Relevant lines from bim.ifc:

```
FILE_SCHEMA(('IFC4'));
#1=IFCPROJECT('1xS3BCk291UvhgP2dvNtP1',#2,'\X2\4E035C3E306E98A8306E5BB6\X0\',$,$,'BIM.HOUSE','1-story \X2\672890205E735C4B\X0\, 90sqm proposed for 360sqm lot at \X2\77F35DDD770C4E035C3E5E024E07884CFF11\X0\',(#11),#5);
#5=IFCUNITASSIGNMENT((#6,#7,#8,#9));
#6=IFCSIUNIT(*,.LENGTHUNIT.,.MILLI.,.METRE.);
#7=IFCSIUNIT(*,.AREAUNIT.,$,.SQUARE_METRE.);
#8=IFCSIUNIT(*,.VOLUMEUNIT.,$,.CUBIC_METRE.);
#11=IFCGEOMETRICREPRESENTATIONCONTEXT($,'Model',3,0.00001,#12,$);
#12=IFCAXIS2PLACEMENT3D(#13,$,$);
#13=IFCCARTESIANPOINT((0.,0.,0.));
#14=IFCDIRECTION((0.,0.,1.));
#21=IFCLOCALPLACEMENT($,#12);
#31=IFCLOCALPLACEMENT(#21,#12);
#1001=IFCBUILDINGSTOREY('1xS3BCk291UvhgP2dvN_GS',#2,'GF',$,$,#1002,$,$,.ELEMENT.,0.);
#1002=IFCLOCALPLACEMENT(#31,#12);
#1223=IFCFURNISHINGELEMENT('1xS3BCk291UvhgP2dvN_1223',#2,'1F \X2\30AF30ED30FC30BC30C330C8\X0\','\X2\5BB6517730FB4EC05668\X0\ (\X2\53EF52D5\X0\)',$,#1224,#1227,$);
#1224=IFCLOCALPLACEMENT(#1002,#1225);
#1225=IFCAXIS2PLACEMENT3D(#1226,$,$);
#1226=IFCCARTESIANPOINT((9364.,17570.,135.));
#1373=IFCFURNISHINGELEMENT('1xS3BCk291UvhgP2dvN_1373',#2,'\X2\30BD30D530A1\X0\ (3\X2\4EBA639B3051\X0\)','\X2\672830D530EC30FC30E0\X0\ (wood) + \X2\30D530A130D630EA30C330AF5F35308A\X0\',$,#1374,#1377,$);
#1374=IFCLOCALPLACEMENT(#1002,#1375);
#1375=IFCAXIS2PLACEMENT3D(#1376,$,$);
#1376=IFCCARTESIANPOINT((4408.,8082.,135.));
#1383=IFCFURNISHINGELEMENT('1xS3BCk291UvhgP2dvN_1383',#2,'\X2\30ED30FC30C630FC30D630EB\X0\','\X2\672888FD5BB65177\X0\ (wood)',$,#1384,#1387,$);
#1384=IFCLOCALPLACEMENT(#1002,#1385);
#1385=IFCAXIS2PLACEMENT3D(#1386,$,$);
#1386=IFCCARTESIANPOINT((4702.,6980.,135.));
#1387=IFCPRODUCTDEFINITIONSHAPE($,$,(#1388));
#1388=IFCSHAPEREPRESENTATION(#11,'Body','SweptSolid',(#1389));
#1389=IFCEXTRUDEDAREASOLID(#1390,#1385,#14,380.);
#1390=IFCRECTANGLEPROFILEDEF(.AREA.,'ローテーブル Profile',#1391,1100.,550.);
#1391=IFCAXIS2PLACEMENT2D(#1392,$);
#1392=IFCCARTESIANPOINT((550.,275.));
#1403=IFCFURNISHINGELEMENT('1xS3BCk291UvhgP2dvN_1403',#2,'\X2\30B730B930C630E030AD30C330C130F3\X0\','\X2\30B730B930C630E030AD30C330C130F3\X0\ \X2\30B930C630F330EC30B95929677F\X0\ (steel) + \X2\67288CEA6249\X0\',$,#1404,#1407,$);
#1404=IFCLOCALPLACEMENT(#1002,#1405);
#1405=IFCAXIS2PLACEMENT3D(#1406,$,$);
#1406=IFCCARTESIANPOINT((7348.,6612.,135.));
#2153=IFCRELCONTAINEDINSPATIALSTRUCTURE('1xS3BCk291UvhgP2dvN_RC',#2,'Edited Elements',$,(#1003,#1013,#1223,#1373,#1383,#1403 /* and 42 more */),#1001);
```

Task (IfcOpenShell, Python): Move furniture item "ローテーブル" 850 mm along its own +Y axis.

```python
import ifcopenshell
import ifcopenshell.api.geometry
import ifcopenshell.util.placement

model = ifcopenshell.open("bim.ifc")

item = model.by_guid("1xS3BCk291UvhgP2dvN_1383")
matrix = ifcopenshell.util.placement.get_local_placement(item.ObjectPlacement)
matrix[:3, 3] += matrix[:3, 1] * 850.0
ifcopenshell.api.geometry.edit_object_placement(model, product=item, matrix=matrix, is_si=False)

print(ifcopenshell.util.placement.get_local_placement(item.ObjectPlacement).round(3) + 0.0)

model.write("bim_v2.ifc")
```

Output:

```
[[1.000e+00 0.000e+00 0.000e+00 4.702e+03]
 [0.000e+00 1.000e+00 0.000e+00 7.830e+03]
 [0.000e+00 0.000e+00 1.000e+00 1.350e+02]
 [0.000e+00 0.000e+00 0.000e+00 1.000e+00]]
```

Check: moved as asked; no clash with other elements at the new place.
